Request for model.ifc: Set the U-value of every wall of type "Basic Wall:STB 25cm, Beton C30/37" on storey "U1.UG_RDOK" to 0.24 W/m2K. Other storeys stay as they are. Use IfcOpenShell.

First a look at what the model holds.

```python
import ifcopenshell
import ifcopenshell.util.element

model = ifcopenshell.open("model.ifc")
print(model.schema)
storey = next(s for s in model.by_type("IfcBuildingStorey") if s.Name == "U1.UG_RDOK")
walls = [e for e in ifcopenshell.util.element.get_decomposition(storey) if e.is_a("IfcWall")]
seen = {}
for e in walls:
    element_type = ifcopenshell.util.element.get_type(e)
    key = (element_type.Name if element_type != e and element_type else None, ifcopenshell.util.element.get_pset(e, "Pset_WallCommon", "ThermalTransmittance"))
    seen[key] = seen.get(key, 0) + 1
for (name, value), count in sorted(seen.items(), key=str):
    print(count, "x", name, "|", value)
```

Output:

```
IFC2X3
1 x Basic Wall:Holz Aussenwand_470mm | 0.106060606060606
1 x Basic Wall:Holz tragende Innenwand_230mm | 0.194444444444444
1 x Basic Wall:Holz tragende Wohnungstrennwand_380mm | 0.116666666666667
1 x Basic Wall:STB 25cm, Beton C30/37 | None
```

```python
import ifcopenshell
import ifcopenshell.api.pset
import ifcopenshell.util.element

model = ifcopenshell.open("model.ifc")

storey = next(s for s in model.by_type("IfcBuildingStorey") if s.Name == "U1.UG_RDOK")
walls = [e for e in ifcopenshell.util.element.get_decomposition(storey) if e.is_a("IfcWall")]

count = 0
for e in walls:
    element_type = ifcopenshell.util.element.get_type(e)
    if element_type in (None, e) or element_type.Name != "Basic Wall:STB 25cm, Beton C30/37":
        continue
    # add_pset returns the element's existing set when there is one.
    pset = ifcopenshell.api.pset.add_pset(model, product=e, name="Pset_WallCommon")
    ifcopenshell.api.pset.edit_pset(model, pset=pset, properties={"ThermalTransmittance": 0.24})
    count += 1

print(count, "walls updated")

model.write("model-out.ifc")
```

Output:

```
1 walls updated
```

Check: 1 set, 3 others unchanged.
